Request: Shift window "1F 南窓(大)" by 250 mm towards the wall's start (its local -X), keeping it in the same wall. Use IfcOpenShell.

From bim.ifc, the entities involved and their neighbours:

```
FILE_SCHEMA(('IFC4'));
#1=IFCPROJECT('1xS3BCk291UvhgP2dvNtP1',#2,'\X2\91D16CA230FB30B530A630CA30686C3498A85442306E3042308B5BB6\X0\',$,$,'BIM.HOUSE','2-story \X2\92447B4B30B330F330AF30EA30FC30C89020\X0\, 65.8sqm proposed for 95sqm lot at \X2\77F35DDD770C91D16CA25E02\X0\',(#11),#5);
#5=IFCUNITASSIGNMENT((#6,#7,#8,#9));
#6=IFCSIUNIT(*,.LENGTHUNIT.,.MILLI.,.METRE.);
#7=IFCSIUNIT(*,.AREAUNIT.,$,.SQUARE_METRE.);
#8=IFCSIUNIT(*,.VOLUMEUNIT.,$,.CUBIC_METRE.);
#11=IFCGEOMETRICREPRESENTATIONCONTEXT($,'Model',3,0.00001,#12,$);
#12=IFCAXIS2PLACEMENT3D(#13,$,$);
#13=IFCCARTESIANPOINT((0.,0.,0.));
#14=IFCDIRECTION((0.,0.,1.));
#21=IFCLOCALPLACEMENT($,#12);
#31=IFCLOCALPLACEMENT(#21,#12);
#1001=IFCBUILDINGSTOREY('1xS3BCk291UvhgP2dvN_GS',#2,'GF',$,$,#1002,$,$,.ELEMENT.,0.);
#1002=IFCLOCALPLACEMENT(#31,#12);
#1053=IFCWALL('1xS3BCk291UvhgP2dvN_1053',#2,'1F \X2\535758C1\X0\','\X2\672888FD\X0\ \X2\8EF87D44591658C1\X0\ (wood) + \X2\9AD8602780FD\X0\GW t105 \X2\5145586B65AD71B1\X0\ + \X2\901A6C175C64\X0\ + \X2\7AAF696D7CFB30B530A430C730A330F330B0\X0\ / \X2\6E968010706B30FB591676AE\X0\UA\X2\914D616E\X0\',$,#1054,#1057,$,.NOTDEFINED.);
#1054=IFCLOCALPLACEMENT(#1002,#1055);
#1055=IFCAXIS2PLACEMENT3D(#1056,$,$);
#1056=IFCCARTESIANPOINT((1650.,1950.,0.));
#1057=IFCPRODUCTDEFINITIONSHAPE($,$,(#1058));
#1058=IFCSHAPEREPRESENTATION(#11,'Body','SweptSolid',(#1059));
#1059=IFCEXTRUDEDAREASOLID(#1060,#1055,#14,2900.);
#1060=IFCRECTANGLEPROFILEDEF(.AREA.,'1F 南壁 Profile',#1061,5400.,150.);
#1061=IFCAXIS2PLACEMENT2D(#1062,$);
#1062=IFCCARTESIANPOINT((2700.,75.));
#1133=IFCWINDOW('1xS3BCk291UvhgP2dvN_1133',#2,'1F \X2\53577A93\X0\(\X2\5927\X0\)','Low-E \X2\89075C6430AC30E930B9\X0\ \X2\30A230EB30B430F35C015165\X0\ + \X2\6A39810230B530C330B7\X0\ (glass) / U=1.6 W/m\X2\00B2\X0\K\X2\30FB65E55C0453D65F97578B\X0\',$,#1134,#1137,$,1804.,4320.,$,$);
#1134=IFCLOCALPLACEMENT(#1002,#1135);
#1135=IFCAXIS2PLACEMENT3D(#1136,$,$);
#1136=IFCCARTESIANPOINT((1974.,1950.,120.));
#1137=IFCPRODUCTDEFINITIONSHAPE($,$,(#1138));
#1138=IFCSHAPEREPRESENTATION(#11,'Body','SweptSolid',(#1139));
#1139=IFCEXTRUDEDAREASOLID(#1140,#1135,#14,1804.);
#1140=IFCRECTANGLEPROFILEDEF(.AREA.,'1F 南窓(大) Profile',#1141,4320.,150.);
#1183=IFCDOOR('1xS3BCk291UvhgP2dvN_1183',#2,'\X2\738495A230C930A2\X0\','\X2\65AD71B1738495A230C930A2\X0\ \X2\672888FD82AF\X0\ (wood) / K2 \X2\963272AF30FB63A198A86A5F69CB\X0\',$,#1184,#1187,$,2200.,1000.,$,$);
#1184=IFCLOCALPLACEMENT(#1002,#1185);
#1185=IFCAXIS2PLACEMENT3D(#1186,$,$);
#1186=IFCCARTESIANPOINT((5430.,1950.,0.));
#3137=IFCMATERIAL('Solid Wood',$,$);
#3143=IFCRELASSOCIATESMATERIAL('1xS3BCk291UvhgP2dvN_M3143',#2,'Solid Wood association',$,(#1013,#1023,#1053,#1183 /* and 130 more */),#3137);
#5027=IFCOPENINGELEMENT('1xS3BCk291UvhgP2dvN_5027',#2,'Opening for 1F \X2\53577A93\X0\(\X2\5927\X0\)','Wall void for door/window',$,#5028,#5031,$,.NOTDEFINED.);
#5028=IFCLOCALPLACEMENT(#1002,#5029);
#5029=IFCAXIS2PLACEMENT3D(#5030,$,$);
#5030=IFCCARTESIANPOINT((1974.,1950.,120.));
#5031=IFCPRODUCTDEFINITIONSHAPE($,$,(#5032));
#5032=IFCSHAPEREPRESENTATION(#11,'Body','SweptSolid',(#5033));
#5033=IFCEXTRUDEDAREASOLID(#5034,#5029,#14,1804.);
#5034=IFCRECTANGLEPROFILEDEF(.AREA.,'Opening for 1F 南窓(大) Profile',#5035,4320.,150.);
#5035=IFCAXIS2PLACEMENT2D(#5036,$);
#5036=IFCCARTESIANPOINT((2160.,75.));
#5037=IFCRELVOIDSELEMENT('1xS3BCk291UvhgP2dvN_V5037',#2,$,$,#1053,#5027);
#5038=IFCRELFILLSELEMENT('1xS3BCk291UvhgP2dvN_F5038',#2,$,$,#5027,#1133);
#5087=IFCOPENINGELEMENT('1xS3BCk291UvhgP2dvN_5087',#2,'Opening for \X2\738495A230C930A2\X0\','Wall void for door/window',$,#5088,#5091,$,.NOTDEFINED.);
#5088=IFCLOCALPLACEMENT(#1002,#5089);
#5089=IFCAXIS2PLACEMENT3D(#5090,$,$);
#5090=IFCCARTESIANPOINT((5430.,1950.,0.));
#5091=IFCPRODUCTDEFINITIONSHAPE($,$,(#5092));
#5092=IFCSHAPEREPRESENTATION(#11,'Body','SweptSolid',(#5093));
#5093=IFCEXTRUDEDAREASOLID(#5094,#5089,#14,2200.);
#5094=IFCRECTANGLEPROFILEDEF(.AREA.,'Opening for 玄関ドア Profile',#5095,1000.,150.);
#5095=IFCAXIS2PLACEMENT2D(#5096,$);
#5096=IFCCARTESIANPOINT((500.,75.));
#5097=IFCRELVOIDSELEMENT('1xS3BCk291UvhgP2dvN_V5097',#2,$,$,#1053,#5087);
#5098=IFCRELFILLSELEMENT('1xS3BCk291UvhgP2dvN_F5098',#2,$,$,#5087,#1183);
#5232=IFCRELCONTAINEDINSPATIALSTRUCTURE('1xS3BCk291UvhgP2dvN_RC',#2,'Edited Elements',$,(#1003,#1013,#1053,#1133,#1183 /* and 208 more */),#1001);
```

```python
import ifcopenshell
import ifcopenshell.api.geometry
import ifcopenshell.util.placement

model = ifcopenshell.open("bim.ifc")

window = model.by_guid("1xS3BCk291UvhgP2dvN_1133")
opening = window.FillsVoids[0].RelatingOpeningElement
wall = opening.VoidsElements[0].RelatingBuildingElement

wall_matrix = ifcopenshell.util.placement.get_local_placement(wall.ObjectPlacement)
shift = wall_matrix[:3, 0] * -250.0
before = ifcopenshell.util.placement.get_local_placement(window.ObjectPlacement)[:3, 3].copy()

# The window is not placed relative to its opening, so move both.
for product in (opening, window):
    matrix = ifcopenshell.util.placement.get_local_placement(product.ObjectPlacement)
    matrix[:3, 3] += shift
    ifcopenshell.api.geometry.edit_object_placement(model, product=product, matrix=matrix, is_si=False)

after = ifcopenshell.util.placement.get_local_placement(window.ObjectPlacement)[:3, 3]
print("window moved by", (after - before).round(3) + 0.0)

model.write("bim_updated.ifc")
```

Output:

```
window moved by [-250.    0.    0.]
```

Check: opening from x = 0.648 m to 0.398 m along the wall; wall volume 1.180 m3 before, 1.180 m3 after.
